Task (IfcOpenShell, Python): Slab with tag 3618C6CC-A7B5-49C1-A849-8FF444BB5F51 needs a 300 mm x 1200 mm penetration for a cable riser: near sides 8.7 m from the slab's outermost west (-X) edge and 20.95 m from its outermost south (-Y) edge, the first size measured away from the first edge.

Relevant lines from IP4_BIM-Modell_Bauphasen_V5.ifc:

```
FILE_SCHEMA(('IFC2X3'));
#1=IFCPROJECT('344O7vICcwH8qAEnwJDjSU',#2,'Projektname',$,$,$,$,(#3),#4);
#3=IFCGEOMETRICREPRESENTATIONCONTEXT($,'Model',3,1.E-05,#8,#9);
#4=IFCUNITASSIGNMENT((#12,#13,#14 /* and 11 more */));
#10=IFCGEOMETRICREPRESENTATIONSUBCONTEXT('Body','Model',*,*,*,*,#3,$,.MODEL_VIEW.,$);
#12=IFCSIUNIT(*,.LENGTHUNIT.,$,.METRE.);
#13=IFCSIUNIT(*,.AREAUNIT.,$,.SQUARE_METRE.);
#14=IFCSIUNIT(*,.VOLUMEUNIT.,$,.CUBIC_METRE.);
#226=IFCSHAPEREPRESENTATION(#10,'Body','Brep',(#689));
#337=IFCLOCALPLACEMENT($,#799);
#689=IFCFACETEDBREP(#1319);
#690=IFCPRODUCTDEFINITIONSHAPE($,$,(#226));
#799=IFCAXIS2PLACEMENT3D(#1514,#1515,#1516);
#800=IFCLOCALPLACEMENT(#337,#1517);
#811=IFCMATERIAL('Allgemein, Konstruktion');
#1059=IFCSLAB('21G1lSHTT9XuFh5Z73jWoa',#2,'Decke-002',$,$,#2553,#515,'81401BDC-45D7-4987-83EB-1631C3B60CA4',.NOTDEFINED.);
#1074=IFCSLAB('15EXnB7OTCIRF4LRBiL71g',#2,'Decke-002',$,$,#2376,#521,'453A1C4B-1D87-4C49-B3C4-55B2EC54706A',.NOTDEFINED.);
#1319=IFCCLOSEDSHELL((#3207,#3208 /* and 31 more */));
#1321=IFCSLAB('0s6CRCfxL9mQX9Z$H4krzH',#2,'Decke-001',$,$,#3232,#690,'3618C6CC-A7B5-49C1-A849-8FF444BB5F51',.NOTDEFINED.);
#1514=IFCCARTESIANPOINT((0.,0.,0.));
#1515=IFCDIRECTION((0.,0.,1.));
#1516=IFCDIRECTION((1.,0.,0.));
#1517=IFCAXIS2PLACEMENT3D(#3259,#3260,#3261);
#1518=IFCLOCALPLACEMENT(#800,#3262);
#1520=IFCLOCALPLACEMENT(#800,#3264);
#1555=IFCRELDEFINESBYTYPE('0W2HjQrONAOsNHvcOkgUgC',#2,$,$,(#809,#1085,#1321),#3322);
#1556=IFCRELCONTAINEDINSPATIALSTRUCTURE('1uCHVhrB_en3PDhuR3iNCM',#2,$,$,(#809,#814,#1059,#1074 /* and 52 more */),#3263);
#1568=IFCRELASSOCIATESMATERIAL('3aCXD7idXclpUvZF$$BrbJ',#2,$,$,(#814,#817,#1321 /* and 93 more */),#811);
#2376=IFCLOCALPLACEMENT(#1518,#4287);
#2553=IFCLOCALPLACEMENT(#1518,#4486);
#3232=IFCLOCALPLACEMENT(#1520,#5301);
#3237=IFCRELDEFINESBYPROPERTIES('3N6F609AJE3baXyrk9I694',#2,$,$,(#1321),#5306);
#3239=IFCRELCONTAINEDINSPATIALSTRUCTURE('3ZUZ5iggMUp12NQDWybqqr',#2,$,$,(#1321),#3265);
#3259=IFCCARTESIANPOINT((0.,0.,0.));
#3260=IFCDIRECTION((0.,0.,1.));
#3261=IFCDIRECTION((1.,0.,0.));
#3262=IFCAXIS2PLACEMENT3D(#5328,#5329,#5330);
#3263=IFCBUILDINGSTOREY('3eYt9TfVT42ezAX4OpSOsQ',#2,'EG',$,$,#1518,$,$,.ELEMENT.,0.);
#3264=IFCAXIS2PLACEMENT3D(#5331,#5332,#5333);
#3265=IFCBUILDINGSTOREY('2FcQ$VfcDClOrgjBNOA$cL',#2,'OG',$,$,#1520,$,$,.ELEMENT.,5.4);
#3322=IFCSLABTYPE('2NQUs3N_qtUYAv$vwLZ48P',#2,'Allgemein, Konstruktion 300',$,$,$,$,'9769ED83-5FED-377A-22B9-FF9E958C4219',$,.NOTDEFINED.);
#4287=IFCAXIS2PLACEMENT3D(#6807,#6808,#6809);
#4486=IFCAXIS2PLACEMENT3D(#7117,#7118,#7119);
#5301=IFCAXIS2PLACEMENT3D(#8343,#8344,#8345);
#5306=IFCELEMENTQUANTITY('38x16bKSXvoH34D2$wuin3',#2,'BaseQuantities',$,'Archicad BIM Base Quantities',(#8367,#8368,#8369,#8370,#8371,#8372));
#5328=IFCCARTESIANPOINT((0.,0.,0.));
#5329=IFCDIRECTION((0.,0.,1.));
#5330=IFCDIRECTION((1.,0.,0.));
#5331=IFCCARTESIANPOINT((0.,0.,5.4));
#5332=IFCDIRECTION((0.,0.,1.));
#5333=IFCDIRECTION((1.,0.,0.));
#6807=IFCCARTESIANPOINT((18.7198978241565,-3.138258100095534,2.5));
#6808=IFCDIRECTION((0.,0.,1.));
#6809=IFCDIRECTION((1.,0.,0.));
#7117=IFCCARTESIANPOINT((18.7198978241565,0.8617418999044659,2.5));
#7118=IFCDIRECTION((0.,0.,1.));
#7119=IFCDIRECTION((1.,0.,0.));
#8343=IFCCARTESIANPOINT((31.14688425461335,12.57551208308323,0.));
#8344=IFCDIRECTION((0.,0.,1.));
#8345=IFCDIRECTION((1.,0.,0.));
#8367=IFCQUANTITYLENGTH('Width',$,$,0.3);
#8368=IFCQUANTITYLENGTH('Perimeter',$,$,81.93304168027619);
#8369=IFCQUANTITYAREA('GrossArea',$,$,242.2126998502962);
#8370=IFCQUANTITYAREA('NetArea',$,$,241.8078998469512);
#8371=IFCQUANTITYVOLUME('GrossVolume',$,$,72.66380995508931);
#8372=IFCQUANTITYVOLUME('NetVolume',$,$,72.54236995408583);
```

```python
import numpy as np
import ifcopenshell
import ifcopenshell.api.feature
import ifcopenshell.api.geometry
import ifcopenshell.api.pset
import ifcopenshell.api.root
import ifcopenshell.geom
import ifcopenshell.util.element
import ifcopenshell.util.placement
import ifcopenshell.util.representation
import ifcopenshell.util.shape
import ifcopenshell.util.unit

model = ifcopenshell.open("IP4_BIM-Modell_Bauphasen_V5.ifc")
unit_scale = ifcopenshell.util.unit.calculate_unit_scale(model)
area_scale = ifcopenshell.util.unit.calculate_unit_scale(model, "AREAUNIT")
volume_scale = ifcopenshell.util.unit.calculate_unit_scale(model, "VOLUMEUNIT")
settings = ifcopenshell.geom.settings()


def volume(element):
    """Net volume in cubic metres, openings subtracted."""
    shape = ifcopenshell.geom.create_shape(settings, element)
    return ifcopenshell.util.shape.get_volume(shape.geometry)


slab = model.by_guid("0s6CRCfxL9mQX9Z$H4krzH")
before = volume(slab)

# Extent in the slab's own axes, in metres. The edges named are its -X and -Y sides.
slab_shape = ifcopenshell.geom.create_shape(settings, slab)
vertices = ifcopenshell.util.shape.get_vertices(slab_shape.geometry)
x_min, y_min, bottom = vertices.min(axis=0)
top = vertices[:, 2].max()

opening = ifcopenshell.api.root.create_entity(model, ifc_class="IfcOpeningElement", name="Cable riser opening")
context = ifcopenshell.util.representation.get_context(model, "Model", "Body", "MODEL_VIEW")
width, depth = 0.3, 1.2
outline = [(0.0, 0.0), (width, 0.0), (width, depth), (0.0, depth), (0.0, 0.0)]
# Overshoot both faces by 50 mm so the cut is clean.
shape = ifcopenshell.api.geometry.add_slab_representation(
    model, context=context, depth=top - bottom + 0.1, polyline=outline
)
ifcopenshell.api.geometry.assign_representation(model, product=opening, representation=shape)

matrix = ifcopenshell.util.placement.get_local_placement(slab.ObjectPlacement)
matrix[:, 3] = matrix @ np.append(np.array([x_min + 8.7, y_min + 20.95, bottom - 0.05]) / unit_scale, 1.0)
ifcopenshell.api.geometry.edit_object_placement(model, product=opening, matrix=matrix, is_si=False)
ifcopenshell.api.feature.add_feature(model, feature=opening, element=slab)

after = volume(slab)

# Update the slab's stored quantities.
qto = model.by_id(ifcopenshell.util.element.get_pset(slab, "BaseQuantities", should_inherit=False)["id"])
ifcopenshell.api.pset.edit_qto(model, qto=qto, properties={
    "NetArea": after / (top - bottom) / area_scale,
    "NetVolume": after / volume_scale,
})

print(f"slab volume {before:.3f} -> {after:.3f} m3")

model.write("IP4_BIM-Modell_Bauphasen_V5_edited.ifc")
```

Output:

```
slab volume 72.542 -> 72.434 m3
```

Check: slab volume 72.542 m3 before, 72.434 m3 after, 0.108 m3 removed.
